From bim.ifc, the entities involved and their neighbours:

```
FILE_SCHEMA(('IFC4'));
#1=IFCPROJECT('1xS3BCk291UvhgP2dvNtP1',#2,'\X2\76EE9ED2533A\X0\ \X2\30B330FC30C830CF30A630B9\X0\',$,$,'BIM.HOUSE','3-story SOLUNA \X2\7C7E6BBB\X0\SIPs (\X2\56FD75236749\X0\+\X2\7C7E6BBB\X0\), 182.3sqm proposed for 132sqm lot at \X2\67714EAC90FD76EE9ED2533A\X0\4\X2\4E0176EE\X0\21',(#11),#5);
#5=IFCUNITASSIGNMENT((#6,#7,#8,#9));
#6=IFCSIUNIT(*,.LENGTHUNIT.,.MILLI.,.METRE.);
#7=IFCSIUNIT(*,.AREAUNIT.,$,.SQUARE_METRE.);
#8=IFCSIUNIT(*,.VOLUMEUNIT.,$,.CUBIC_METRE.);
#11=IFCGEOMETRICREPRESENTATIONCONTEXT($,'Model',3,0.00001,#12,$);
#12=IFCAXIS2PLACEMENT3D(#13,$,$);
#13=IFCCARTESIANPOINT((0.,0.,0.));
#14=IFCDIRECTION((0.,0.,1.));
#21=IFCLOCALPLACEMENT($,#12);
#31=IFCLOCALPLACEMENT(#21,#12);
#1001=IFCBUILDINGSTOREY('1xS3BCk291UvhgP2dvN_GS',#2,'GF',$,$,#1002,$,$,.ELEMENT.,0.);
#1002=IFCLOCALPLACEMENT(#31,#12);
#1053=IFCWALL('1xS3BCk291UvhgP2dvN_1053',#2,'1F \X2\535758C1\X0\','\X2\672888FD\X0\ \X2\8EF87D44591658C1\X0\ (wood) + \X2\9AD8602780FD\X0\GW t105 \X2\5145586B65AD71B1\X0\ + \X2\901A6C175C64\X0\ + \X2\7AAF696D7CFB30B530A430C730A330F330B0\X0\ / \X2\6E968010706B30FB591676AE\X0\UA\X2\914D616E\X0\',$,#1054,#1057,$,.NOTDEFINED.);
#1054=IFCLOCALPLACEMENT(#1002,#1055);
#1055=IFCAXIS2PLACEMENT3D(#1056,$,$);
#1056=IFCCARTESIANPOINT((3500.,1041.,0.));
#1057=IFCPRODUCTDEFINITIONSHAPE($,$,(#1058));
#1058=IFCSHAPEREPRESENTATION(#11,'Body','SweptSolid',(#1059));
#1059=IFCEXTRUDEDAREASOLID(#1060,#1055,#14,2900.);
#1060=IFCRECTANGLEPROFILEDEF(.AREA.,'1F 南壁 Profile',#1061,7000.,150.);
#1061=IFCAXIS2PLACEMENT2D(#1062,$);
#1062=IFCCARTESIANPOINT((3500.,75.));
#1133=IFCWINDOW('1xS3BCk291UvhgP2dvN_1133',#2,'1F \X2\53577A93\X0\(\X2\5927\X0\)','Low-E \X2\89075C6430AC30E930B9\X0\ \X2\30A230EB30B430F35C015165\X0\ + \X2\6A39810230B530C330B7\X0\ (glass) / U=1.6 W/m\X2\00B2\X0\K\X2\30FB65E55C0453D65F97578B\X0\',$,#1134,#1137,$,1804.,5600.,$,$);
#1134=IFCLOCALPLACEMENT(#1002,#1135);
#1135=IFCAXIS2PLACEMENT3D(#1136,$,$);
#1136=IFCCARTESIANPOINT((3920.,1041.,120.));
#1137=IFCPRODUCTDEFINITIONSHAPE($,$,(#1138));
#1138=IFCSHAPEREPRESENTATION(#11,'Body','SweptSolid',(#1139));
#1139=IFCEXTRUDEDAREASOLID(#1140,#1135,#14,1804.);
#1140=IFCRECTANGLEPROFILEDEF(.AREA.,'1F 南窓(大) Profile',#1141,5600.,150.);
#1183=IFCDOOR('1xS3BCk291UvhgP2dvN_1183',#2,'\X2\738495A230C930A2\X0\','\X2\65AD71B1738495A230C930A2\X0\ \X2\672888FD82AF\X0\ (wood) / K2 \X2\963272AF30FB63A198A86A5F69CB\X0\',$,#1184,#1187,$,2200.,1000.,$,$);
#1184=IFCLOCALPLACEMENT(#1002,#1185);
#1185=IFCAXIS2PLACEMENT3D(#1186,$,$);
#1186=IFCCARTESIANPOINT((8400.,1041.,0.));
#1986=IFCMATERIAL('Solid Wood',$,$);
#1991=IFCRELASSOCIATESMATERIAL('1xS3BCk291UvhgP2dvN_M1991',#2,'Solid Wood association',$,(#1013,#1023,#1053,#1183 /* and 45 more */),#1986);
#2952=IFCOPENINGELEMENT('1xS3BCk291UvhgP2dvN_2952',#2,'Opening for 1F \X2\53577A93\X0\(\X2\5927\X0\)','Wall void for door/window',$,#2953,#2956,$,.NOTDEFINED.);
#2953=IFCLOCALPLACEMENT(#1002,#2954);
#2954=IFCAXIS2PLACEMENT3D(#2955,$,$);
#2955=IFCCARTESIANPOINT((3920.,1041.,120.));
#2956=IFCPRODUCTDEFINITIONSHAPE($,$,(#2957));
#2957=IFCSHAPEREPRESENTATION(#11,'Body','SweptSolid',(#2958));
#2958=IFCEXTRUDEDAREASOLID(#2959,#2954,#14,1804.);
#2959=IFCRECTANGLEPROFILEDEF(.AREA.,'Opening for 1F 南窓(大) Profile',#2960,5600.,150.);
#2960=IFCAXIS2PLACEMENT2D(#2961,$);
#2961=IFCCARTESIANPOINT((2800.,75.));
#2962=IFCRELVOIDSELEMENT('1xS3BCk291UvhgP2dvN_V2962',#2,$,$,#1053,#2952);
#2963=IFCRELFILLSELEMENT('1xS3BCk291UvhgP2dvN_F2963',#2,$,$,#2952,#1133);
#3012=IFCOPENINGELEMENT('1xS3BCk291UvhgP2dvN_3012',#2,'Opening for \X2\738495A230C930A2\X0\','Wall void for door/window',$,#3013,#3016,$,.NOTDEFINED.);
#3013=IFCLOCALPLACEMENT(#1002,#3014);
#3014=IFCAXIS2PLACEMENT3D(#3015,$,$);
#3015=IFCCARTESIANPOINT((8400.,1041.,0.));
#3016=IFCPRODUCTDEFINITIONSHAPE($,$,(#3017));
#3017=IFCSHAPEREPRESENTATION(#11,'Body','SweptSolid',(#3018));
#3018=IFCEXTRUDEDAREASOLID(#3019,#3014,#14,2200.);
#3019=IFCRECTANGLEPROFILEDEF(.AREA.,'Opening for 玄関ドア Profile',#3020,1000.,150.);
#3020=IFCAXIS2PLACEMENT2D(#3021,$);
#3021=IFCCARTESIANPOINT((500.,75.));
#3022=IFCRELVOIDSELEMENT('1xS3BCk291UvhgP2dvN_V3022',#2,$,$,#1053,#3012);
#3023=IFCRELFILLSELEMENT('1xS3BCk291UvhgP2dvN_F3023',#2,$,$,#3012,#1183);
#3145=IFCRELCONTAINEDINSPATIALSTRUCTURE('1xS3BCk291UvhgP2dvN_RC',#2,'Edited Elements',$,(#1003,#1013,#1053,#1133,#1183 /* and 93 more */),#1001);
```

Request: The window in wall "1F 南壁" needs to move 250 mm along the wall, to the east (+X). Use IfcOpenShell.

```python
import ifcopenshell
import ifcopenshell.api.geometry
import ifcopenshell.util.placement
import ifcopenshell.util.unit

model = ifcopenshell.open("bim.ifc")
unit_scale = ifcopenshell.util.unit.calculate_unit_scale(model)

window = model.by_id(1133)
opening = window.FillsVoids[0].RelatingOpeningElement
wall = opening.VoidsElements[0].RelatingBuildingElement

wall_matrix = ifcopenshell.util.placement.get_local_placement(wall.ObjectPlacement)
shift = wall_matrix[:3, 0] * 0.25 / unit_scale
before = ifcopenshell.util.placement.get_local_placement(window.ObjectPlacement)[:3, 3].copy()

# The window is not placed relative to its opening, so move both.
for product in (opening, window):
    matrix = ifcopenshell.util.placement.get_local_placement(product.ObjectPlacement)
    matrix[:3, 3] += shift
    ifcopenshell.api.geometry.edit_object_placement(model, product=product, matrix=matrix, is_si=False)

after = ifcopenshell.util.placement.get_local_placement(window.ObjectPlacement)[:3, 3]
print("window moved by", (after - before).round(3) + 0.0)

model.write("bim_rev.ifc")
```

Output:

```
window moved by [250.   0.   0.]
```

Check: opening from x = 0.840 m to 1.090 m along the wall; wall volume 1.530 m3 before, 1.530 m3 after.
